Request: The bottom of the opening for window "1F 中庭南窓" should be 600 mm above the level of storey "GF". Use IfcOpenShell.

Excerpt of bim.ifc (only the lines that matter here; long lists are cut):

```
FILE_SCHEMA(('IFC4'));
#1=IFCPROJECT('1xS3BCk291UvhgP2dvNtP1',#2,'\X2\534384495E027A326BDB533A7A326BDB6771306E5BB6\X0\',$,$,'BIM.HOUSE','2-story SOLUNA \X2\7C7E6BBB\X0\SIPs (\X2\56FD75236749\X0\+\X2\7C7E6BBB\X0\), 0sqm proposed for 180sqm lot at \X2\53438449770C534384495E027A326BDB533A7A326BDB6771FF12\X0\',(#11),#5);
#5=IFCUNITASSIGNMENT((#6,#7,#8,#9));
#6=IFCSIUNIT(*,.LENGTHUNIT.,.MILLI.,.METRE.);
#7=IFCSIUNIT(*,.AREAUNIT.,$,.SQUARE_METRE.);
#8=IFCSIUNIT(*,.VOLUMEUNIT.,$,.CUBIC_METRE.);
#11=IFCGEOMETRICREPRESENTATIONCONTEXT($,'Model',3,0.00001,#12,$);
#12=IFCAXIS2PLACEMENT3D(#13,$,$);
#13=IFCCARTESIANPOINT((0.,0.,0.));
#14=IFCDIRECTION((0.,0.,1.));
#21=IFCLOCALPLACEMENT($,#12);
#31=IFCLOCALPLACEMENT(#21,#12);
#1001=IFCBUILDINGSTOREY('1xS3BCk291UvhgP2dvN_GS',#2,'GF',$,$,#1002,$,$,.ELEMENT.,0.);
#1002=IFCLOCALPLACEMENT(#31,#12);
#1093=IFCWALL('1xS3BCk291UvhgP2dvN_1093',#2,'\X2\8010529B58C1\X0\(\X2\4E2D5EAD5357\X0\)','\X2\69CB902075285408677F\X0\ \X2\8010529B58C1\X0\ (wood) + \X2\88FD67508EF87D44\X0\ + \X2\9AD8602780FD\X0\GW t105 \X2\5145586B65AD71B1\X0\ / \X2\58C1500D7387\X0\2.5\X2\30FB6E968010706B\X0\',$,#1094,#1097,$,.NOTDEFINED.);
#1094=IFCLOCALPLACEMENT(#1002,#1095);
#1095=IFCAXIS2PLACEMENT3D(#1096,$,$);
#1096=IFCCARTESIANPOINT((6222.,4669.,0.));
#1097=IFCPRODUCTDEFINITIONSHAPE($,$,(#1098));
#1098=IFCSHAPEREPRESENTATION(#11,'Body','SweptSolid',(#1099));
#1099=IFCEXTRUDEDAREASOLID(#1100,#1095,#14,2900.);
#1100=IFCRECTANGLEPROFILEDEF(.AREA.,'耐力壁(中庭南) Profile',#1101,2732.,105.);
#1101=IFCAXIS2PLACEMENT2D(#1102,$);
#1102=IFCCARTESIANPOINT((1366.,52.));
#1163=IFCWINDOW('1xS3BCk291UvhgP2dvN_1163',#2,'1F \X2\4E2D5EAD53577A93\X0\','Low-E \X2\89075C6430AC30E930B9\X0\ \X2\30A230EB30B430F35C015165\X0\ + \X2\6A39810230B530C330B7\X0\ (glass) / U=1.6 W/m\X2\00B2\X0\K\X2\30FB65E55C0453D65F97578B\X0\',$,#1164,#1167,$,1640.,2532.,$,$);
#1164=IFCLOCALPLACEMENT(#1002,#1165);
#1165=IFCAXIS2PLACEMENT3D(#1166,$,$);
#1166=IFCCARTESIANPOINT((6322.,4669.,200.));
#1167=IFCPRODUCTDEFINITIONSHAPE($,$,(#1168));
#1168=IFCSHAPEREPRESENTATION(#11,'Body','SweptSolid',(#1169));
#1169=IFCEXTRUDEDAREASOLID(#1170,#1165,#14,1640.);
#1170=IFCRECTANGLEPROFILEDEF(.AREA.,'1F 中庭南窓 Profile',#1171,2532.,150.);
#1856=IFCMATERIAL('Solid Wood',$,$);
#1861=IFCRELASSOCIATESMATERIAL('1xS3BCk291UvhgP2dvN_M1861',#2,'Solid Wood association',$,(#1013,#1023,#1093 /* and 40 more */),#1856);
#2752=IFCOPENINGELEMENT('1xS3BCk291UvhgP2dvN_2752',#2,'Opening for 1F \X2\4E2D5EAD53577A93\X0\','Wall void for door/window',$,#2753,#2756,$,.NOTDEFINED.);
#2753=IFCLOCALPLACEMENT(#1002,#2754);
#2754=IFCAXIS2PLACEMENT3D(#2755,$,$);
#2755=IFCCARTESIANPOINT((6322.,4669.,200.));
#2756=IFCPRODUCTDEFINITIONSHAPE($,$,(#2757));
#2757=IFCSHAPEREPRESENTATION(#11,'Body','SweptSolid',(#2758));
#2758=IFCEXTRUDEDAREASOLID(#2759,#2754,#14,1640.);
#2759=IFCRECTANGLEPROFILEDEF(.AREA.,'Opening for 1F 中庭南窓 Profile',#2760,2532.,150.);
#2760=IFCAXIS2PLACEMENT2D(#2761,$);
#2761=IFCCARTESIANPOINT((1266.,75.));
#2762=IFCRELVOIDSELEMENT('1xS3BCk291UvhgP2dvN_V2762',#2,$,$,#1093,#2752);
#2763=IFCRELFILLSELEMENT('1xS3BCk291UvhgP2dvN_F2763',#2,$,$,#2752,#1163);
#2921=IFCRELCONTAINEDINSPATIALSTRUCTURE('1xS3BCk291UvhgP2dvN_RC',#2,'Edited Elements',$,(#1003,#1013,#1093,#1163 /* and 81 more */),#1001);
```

```python
import numpy as np
import ifcopenshell
import ifcopenshell.api.geometry
import ifcopenshell.geom
import ifcopenshell.util.element
import ifcopenshell.util.placement
import ifcopenshell.util.shape
import ifcopenshell.util.unit

model = ifcopenshell.open("bim.ifc")
unit_scale = ifcopenshell.util.unit.calculate_unit_scale(model)

window = model.by_guid("1xS3BCk291UvhgP2dvN_1163")
opening = window.FillsVoids[0].RelatingOpeningElement
storey = ifcopenshell.util.element.get_container(window, ifc_class="IfcBuildingStorey")
level = ifcopenshell.util.placement.get_local_placement(storey.ObjectPlacement)[2, 3]

# The opening's origin need not be at the sill, so measure its lowest point.
shape = ifcopenshell.geom.create_shape(ifcopenshell.geom.settings(), opening)
bottom = ifcopenshell.util.shape.get_shape_bottom_elevation(shape, shape.geometry) / unit_scale
dz = level + 0.6 / unit_scale - bottom

shift = np.array([0.0, 0.0, dz])
# The window is not placed relative to its opening, so move both.
for product in (opening, window):
    matrix = ifcopenshell.util.placement.get_local_placement(product.ObjectPlacement)
    matrix[:3, 3] += shift
    ifcopenshell.api.geometry.edit_object_placement(model, product=product, matrix=matrix, is_si=False)

print(f"moved by {dz * unit_scale:+.3f} m")

model.write("bim_v2.ifc")
```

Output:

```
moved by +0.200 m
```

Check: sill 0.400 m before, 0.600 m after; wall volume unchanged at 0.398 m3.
